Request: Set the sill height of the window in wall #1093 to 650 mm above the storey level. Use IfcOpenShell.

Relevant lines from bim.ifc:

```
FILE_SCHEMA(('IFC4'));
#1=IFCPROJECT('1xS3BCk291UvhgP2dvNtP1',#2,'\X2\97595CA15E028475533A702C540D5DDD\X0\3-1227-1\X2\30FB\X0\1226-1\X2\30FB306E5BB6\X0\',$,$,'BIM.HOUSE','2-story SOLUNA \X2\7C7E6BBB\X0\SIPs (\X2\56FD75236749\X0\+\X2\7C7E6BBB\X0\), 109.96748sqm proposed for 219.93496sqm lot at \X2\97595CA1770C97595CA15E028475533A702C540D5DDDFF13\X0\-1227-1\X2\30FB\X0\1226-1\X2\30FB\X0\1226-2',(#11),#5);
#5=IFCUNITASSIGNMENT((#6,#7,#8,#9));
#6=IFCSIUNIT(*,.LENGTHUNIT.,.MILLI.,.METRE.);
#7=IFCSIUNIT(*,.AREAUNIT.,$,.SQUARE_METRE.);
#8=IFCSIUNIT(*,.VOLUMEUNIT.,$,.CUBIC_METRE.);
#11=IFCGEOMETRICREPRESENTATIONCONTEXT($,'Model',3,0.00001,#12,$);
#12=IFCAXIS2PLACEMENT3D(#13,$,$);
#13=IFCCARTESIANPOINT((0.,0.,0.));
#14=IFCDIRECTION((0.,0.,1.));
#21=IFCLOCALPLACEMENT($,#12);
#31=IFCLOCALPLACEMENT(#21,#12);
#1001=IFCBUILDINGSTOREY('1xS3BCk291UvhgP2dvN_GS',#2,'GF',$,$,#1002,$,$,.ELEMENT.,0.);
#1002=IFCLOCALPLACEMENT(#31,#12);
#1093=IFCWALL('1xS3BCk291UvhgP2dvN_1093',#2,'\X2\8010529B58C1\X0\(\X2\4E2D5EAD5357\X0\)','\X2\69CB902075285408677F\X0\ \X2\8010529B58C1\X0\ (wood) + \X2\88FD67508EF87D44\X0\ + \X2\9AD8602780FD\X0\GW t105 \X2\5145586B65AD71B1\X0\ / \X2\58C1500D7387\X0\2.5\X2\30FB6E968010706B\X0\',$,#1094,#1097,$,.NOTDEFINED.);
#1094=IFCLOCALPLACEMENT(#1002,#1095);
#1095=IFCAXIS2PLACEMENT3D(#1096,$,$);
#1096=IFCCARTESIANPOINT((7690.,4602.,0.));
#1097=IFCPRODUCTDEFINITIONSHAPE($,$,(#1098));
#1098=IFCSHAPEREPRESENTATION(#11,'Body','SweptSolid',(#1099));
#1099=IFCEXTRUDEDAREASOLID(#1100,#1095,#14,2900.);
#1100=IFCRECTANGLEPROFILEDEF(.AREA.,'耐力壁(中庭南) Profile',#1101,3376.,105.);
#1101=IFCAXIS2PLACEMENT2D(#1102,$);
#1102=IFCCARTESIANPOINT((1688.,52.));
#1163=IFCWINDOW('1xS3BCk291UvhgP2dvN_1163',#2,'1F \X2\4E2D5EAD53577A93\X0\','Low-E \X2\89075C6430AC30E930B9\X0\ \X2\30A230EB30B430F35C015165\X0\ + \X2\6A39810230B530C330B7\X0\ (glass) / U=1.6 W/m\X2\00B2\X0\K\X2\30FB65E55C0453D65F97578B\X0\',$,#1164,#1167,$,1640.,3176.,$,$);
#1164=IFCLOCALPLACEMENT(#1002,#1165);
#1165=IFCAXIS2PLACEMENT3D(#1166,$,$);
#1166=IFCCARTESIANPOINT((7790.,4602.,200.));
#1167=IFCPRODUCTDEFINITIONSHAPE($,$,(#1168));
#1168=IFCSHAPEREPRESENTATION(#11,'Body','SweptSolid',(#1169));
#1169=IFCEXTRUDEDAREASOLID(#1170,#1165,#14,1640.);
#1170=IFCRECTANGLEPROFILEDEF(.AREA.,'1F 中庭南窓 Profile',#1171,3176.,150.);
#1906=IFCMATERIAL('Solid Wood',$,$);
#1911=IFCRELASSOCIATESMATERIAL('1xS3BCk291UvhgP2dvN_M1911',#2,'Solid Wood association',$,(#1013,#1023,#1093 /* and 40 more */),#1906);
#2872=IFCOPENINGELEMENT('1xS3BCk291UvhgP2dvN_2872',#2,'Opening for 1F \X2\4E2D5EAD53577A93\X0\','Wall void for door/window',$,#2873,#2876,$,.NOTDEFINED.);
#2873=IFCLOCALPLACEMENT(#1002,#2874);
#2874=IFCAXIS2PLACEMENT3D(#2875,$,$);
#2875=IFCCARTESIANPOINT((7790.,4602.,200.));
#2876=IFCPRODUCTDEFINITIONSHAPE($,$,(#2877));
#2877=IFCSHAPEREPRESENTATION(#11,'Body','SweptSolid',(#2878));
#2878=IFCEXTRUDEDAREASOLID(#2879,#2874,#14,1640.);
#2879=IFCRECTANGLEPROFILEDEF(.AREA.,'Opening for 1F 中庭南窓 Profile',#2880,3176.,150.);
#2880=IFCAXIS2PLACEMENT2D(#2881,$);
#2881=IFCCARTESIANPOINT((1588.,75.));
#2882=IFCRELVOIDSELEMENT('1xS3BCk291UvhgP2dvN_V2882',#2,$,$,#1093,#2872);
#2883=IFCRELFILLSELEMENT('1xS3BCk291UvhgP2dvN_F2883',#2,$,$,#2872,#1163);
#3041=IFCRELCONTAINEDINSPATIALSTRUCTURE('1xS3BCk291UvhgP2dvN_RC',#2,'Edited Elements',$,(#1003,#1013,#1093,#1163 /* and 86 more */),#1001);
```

```python
import numpy as np
import ifcopenshell
import ifcopenshell.api.geometry
import ifcopenshell.geom
import ifcopenshell.util.element
import ifcopenshell.util.placement
import ifcopenshell.util.shape
import ifcopenshell.util.unit

model = ifcopenshell.open("bim.ifc")
unit_scale = ifcopenshell.util.unit.calculate_unit_scale(model)

window = model.by_id(1163)
opening = window.FillsVoids[0].RelatingOpeningElement
storey = ifcopenshell.util.element.get_container(window, ifc_class="IfcBuildingStorey")
level = ifcopenshell.util.placement.get_local_placement(storey.ObjectPlacement)[2, 3]

# The opening's origin need not be at the sill, so measure its lowest point.
shape = ifcopenshell.geom.create_shape(ifcopenshell.geom.settings(), opening)
bottom = ifcopenshell.util.shape.get_shape_bottom_elevation(shape, shape.geometry) / unit_scale
dz = level + 0.65 / unit_scale - bottom

shift = np.array([0.0, 0.0, dz])
# The window is not placed relative to its opening, so move both.
for product in (opening, window):
    matrix = ifcopenshell.util.placement.get_local_placement(product.ObjectPlacement)
    matrix[:3, 3] += shift
    ifcopenshell.api.geometry.edit_object_placement(model, product=product, matrix=matrix, is_si=False)

print(f"moved by {dz * unit_scale:+.3f} m")

model.write("bim-out.ifc")
```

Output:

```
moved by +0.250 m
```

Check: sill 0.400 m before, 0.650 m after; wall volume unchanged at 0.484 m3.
